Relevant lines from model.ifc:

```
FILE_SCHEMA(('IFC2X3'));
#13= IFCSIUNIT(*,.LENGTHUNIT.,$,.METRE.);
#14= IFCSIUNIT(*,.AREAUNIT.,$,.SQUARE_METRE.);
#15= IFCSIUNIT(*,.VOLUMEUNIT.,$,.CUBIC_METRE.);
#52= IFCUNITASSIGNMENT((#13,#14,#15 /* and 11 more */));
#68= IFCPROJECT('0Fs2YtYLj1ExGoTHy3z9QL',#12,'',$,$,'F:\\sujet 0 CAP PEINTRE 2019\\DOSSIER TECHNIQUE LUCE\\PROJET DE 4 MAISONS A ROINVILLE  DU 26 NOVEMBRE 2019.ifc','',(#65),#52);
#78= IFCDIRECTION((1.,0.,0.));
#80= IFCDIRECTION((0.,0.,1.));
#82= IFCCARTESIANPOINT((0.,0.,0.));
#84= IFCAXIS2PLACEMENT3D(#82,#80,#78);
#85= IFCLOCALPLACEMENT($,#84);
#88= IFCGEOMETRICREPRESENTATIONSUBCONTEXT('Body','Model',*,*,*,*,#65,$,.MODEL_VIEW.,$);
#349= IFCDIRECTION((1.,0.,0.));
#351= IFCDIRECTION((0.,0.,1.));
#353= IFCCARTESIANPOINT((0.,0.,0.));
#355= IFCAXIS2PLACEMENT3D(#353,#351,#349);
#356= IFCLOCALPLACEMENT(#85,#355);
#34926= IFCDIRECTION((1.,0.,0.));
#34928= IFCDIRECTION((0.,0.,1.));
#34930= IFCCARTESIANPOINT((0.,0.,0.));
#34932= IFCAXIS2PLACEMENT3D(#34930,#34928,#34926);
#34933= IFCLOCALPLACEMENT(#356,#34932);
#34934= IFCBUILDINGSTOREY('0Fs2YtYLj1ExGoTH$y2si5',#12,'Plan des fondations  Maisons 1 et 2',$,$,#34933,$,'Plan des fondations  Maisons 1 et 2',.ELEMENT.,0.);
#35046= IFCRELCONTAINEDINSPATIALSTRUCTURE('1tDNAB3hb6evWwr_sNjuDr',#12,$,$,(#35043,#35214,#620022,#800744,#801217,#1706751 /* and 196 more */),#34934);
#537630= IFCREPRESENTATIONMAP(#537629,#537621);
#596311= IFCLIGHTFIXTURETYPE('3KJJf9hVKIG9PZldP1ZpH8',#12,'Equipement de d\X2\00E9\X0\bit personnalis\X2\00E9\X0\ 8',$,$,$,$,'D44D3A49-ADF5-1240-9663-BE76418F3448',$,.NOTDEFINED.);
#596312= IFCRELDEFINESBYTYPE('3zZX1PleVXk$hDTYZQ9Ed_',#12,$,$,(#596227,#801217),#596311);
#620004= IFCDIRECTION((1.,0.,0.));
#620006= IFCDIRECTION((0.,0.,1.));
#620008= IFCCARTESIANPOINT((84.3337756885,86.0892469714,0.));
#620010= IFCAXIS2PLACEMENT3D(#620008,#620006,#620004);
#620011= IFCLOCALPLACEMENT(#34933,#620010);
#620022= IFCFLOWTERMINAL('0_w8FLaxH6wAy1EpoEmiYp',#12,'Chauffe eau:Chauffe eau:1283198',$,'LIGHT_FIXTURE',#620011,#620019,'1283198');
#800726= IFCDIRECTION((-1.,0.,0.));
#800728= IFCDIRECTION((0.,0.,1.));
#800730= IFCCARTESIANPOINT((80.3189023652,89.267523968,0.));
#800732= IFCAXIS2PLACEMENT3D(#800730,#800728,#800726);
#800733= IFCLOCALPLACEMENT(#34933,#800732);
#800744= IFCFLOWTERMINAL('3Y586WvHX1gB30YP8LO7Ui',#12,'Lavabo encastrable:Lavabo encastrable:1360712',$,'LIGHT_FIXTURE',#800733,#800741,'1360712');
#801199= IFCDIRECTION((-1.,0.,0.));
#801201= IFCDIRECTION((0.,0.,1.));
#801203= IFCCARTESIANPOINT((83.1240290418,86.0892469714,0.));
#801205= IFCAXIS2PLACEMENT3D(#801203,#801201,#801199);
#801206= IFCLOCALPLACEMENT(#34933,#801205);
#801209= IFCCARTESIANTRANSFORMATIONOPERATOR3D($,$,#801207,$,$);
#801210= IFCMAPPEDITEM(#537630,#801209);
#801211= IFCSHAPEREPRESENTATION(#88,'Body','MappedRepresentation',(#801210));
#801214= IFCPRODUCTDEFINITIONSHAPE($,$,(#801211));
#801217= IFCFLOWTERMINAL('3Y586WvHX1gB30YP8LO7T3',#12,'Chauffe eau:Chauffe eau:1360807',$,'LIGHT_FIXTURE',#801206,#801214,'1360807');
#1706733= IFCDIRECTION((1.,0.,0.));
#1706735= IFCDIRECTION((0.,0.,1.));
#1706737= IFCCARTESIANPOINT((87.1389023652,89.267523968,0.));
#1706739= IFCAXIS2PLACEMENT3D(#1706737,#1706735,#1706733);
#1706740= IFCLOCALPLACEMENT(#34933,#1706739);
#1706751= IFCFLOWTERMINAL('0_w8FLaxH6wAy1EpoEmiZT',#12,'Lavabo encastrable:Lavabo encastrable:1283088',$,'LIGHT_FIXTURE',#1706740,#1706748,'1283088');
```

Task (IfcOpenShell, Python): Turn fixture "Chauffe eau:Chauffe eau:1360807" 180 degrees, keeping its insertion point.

```python
import ifcopenshell
import ifcopenshell.api.geometry
import ifcopenshell.util.placement

model = ifcopenshell.open("model.ifc")

item = model.by_guid("3Y586WvHX1gB30YP8LO7T3")
matrix = ifcopenshell.util.placement.get_local_placement(item.ObjectPlacement)
matrix = matrix @ ifcopenshell.util.placement.rotation(180, "Z")
ifcopenshell.api.geometry.edit_object_placement(model, product=item, matrix=matrix, is_si=False)

print(ifcopenshell.util.placement.get_local_placement(item.ObjectPlacement).round(3) + 0.0)

model.write("model_edited.ifc")
```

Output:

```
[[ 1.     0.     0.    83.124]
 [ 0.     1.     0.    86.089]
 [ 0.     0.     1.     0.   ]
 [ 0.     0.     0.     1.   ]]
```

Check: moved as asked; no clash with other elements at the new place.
